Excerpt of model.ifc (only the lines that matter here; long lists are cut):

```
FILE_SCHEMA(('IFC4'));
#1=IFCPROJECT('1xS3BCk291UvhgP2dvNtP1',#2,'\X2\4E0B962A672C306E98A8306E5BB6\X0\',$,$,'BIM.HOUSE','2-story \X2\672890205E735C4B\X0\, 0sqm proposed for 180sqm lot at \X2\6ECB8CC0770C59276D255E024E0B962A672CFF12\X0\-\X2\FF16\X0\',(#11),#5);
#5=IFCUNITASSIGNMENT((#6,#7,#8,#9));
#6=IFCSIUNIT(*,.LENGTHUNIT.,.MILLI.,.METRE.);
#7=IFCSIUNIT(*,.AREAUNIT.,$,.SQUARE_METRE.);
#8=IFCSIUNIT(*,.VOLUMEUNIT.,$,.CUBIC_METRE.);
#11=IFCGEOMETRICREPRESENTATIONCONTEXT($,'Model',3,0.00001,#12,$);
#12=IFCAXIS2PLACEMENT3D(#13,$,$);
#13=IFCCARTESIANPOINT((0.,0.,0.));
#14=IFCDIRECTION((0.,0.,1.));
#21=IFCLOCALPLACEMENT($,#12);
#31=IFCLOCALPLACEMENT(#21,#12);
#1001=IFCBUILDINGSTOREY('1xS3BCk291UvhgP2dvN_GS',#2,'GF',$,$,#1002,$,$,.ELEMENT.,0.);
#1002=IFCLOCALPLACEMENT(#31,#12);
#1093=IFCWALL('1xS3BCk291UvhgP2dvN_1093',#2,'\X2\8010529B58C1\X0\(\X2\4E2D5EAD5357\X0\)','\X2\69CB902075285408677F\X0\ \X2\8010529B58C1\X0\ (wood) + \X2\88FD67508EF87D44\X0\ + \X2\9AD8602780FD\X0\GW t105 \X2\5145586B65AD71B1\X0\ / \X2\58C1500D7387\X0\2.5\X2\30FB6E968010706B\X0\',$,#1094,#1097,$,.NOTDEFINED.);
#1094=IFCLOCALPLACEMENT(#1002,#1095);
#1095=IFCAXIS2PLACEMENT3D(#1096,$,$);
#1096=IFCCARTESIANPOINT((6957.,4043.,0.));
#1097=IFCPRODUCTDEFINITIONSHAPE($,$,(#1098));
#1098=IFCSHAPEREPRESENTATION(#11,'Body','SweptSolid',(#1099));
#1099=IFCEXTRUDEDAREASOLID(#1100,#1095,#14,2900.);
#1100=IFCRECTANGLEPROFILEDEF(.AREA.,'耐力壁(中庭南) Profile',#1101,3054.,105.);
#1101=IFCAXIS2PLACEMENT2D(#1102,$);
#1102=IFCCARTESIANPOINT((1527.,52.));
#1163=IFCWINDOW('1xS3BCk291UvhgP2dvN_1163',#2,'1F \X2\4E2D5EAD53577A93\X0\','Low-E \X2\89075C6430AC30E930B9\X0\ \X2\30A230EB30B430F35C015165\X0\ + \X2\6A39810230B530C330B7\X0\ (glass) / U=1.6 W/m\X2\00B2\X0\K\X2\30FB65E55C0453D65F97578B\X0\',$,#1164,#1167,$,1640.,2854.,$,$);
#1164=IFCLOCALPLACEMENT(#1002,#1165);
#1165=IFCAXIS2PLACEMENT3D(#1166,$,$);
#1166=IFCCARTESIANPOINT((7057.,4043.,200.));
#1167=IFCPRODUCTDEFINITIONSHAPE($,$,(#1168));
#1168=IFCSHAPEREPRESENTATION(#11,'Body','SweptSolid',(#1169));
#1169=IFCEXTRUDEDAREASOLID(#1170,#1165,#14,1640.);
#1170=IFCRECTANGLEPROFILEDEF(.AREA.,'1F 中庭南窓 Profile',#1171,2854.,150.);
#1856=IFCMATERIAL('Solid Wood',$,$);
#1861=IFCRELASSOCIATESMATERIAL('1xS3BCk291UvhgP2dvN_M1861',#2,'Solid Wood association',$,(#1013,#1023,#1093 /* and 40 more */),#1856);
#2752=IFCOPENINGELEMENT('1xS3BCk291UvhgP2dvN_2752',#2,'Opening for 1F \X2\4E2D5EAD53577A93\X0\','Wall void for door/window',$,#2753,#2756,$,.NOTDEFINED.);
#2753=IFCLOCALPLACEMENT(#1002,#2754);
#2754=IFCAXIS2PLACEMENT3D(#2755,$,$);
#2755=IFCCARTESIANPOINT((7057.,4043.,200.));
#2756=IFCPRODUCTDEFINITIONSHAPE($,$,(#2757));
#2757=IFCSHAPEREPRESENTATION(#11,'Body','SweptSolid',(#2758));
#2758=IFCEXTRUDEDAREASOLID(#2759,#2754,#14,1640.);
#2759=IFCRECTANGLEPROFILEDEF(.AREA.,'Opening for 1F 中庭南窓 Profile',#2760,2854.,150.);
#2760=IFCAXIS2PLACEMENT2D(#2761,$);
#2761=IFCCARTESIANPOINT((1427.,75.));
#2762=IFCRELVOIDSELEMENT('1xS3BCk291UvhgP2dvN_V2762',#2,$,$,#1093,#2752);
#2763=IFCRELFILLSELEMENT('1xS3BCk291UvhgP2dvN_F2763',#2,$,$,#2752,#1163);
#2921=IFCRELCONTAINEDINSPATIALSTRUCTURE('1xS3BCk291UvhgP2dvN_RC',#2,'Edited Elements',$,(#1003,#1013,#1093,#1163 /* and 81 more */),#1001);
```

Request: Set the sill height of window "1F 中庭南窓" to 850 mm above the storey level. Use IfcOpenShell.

```python
import numpy as np
import ifcopenshell
import ifcopenshell.api.geometry
import ifcopenshell.geom
import ifcopenshell.util.element
import ifcopenshell.util.placement
import ifcopenshell.util.shape
import ifcopenshell.util.unit

model = ifcopenshell.open("model.ifc")
unit_scale = ifcopenshell.util.unit.calculate_unit_scale(model)

window = model.by_guid("1xS3BCk291UvhgP2dvN_1163")
opening = window.FillsVoids[0].RelatingOpeningElement
storey = ifcopenshell.util.element.get_container(window, ifc_class="IfcBuildingStorey")
level = ifcopenshell.util.placement.get_local_placement(storey.ObjectPlacement)[2, 3]

# The opening's origin need not be at the sill, so measure its lowest point.
shape = ifcopenshell.geom.create_shape(ifcopenshell.geom.settings(), opening)
bottom = ifcopenshell.util.shape.get_shape_bottom_elevation(shape, shape.geometry) / unit_scale
dz = level + 850.0 - bottom

shift = np.array([0.0, 0.0, dz])
# The window is not placed relative to its opening, so move both.
for product in (opening, window):
    matrix = ifcopenshell.util.placement.get_local_placement(product.ObjectPlacement)
    matrix[:3, 3] += shift
    ifcopenshell.api.geometry.edit_object_placement(model, product=product, matrix=matrix, is_si=False)

print(f"moved by {dz * unit_scale:+.3f} m")

model.write("model_edited.ifc")
```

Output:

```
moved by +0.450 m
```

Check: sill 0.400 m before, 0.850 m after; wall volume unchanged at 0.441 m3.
